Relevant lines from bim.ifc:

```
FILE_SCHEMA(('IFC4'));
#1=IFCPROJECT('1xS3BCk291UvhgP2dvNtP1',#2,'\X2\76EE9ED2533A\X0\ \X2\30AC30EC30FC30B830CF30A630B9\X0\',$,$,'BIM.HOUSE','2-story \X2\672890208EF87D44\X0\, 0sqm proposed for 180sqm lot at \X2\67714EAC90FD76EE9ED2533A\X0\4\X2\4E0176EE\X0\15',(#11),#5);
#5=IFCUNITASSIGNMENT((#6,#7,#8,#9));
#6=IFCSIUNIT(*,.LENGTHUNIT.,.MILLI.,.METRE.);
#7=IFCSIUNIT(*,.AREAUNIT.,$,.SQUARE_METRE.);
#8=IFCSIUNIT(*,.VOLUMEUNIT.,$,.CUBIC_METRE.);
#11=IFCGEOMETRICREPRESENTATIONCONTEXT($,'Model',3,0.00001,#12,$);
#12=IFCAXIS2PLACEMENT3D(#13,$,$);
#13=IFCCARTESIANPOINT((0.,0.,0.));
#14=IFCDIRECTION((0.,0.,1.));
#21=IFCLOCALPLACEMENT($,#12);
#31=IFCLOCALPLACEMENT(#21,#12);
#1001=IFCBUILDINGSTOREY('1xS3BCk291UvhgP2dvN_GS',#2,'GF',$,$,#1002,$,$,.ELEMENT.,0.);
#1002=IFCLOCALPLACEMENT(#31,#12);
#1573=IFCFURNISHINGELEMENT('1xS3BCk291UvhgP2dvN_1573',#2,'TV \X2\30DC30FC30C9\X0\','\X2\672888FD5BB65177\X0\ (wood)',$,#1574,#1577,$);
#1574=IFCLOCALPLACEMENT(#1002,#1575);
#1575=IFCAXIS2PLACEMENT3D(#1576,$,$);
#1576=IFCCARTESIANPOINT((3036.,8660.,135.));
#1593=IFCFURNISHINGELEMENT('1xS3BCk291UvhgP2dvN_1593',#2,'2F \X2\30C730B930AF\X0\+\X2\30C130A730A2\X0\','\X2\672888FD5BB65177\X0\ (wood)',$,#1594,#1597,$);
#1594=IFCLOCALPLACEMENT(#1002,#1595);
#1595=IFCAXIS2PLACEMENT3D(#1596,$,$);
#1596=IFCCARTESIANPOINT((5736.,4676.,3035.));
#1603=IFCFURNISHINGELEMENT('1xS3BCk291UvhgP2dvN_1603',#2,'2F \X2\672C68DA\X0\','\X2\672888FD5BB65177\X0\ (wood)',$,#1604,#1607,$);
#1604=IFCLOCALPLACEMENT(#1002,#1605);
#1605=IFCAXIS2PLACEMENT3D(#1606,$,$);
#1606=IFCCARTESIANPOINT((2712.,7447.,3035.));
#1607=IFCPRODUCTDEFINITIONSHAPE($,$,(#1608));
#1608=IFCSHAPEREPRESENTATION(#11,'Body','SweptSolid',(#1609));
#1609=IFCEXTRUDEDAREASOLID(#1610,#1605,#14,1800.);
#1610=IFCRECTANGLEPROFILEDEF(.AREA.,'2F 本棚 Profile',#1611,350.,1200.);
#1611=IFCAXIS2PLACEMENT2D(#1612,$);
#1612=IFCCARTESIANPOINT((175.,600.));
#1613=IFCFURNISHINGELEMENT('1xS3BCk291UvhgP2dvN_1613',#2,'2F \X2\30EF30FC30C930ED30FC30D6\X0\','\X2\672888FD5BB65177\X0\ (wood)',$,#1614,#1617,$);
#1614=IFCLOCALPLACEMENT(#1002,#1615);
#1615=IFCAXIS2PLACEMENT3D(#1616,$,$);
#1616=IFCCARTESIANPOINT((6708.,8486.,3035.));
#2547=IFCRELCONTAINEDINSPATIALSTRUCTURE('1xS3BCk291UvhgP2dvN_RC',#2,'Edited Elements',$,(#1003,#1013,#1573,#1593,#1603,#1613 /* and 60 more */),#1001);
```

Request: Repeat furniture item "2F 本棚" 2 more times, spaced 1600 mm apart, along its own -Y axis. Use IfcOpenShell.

```python
import ifcopenshell
import ifcopenshell.api.geometry
import ifcopenshell.api.root
import ifcopenshell.util.element
import ifcopenshell.util.placement
import ifcopenshell.util.unit

model = ifcopenshell.open("bim.ifc")
unit_scale = ifcopenshell.util.unit.calculate_unit_scale(model)


def reuse_history(source, copy):
    """copy_class also copies each property set's owner history, people and application; keep the originals."""
    for rel in copy.IsDefinedBy:
        if rel.is_a("IfcRelDefinesByProperties") and (history := rel.RelatingPropertyDefinition.OwnerHistory):
            rel.RelatingPropertyDefinition.OwnerHistory = source.OwnerHistory
            ifcopenshell.util.element.remove_deep2(model, history)


source = model.by_guid("1xS3BCk291UvhgP2dvN_1603")
base = ifcopenshell.util.placement.get_local_placement(source.ObjectPlacement)
step = -base[:3, 1] * 1.6 / unit_scale

for i in range(1, 3):
    copy = ifcopenshell.api.root.copy_class(model, product=source)
    copy.Representation = ifcopenshell.util.element.copy_deep(
        model, source.Representation, exclude=["IfcGeometricRepresentationContext", "IfcRepresentationMap"]
    )
    reuse_history(source, copy)
    matrix = base.copy()
    matrix[:3, 3] += i * step
    print("added at", matrix[:3, 3].round(3) + 0.0)
    ifcopenshell.api.geometry.edit_object_placement(model, product=copy, matrix=matrix, is_si=False)

model.write("bim_v2.ifc")
```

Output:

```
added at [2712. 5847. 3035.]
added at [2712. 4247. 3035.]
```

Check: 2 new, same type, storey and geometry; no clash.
